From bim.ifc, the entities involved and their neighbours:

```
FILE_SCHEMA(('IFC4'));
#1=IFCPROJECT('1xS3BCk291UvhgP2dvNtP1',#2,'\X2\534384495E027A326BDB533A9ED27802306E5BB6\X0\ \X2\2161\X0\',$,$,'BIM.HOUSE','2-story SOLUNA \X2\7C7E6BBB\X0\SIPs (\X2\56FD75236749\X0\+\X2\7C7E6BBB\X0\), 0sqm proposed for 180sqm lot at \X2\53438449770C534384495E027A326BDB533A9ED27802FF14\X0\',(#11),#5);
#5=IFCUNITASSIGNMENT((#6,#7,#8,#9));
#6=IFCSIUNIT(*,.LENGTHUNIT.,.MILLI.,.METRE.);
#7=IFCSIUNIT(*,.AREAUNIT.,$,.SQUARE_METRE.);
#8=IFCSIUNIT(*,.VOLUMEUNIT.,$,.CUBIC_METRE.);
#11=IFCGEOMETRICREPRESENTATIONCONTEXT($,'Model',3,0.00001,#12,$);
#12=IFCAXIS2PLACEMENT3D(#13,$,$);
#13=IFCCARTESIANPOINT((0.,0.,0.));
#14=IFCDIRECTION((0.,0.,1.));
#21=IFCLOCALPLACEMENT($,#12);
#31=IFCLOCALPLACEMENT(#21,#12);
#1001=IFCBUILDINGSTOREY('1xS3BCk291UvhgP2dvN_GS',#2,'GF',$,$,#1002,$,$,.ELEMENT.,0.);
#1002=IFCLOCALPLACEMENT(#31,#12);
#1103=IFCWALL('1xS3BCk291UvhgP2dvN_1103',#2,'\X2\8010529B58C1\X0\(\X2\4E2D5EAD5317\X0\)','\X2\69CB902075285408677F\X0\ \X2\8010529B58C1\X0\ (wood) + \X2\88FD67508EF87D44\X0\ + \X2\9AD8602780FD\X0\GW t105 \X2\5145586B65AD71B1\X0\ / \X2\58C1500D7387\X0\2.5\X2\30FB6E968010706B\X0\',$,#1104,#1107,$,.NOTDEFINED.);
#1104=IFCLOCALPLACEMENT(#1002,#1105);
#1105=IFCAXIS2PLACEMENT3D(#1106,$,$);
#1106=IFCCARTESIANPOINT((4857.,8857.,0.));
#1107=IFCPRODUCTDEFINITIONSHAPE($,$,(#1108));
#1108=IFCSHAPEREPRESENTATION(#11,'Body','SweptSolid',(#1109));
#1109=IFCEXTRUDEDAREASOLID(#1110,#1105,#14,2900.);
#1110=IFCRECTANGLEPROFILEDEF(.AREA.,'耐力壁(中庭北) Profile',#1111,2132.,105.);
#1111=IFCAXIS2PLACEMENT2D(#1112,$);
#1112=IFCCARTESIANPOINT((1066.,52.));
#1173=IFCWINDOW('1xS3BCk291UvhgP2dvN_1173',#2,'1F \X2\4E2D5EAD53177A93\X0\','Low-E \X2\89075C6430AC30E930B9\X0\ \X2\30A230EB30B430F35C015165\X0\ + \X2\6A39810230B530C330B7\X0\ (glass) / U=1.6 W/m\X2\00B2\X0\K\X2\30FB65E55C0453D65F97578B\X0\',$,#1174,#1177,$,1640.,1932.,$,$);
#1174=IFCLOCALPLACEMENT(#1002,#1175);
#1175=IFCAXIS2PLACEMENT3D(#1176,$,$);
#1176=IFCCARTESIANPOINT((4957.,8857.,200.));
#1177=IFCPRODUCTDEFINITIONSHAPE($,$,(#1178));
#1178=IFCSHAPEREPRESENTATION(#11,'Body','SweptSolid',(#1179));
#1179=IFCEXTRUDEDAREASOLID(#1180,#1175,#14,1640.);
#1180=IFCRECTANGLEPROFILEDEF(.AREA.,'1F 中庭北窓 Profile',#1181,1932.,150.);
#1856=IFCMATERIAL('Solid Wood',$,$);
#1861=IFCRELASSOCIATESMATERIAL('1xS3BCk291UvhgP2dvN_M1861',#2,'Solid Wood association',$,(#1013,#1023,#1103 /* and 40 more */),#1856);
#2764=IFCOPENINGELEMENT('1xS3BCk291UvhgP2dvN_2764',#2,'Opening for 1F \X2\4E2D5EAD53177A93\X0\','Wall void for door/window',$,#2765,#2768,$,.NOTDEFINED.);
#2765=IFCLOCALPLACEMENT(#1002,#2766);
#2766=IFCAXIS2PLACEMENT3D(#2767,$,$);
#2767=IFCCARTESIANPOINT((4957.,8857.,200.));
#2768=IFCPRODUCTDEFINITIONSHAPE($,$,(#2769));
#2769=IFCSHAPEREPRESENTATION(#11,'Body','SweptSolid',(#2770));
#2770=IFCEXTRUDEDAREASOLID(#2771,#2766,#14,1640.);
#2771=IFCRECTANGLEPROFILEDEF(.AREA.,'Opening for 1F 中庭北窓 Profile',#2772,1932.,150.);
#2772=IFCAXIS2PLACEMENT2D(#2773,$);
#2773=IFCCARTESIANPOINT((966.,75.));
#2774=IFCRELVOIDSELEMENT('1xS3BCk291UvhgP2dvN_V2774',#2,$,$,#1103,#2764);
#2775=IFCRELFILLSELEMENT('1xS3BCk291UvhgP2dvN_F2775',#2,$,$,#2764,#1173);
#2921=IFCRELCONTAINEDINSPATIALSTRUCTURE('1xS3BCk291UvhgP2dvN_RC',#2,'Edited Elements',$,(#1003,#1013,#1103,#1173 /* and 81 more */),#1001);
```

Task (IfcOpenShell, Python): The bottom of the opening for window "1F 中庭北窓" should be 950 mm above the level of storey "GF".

```python
import numpy as np
import ifcopenshell
import ifcopenshell.api.geometry
import ifcopenshell.geom
import ifcopenshell.util.element
import ifcopenshell.util.placement
import ifcopenshell.util.shape
import ifcopenshell.util.unit

model = ifcopenshell.open("bim.ifc")
unit_scale = ifcopenshell.util.unit.calculate_unit_scale(model)

window = model.by_guid("1xS3BCk291UvhgP2dvN_1173")
opening = window.FillsVoids[0].RelatingOpeningElement
storey = ifcopenshell.util.element.get_container(window, ifc_class="IfcBuildingStorey")
level = ifcopenshell.util.placement.get_local_placement(storey.ObjectPlacement)[2, 3]

# The opening's origin need not be at the sill, so measure its lowest point.
shape = ifcopenshell.geom.create_shape(ifcopenshell.geom.settings(), opening)
bottom = ifcopenshell.util.shape.get_shape_bottom_elevation(shape, shape.geometry) / unit_scale
dz = level + 0.95 / unit_scale - bottom

shift = np.array([0.0, 0.0, dz])
# The window is not placed relative to its opening, so move both.
for product in (opening, window):
    matrix = ifcopenshell.util.placement.get_local_placement(product.ObjectPlacement)
    matrix[:3, 3] += shift
    ifcopenshell.api.geometry.edit_object_placement(model, product=product, matrix=matrix, is_si=False)

print(f"moved by {dz * unit_scale:+.3f} m")

model.write("bim_v2.ifc")
```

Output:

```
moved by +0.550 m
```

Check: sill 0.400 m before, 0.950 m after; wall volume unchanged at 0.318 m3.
